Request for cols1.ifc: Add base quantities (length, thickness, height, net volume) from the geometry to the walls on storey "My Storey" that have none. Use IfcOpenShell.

First a look at what the model holds.

```python
import ifcopenshell
import ifcopenshell.util.element
import ifcopenshell.util.unit

model = ifcopenshell.open("cols1.ifc")
print(model.schema)
for unit_type in ("LENGTHUNIT", "AREAUNIT", "VOLUMEUNIT"):
    print(unit_type, ifcopenshell.util.unit.calculate_unit_scale(model, unit_type))
storey = next(s for s in model.by_type("IfcBuildingStorey") if s.Name == "My Storey")
walls = [e for e in ifcopenshell.util.element.get_decomposition(storey) if e.is_a("IfcWall")]
for e in sorted(walls, key=lambda e: e.id()):
    print(e.id(), e.is_a(), e.Name, list(ifcopenshell.util.element.get_psets(e, qtos_only=True)), sep=" | ")
```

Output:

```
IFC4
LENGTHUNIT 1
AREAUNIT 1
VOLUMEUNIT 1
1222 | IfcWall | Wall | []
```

```python
import ifcopenshell
import ifcopenshell.api.pset
import ifcopenshell.geom
import ifcopenshell.util.element
import ifcopenshell.util.shape
import ifcopenshell.util.unit

model = ifcopenshell.open("cols1.ifc")
unit_scale = ifcopenshell.util.unit.calculate_unit_scale(model)
volume_scale = ifcopenshell.util.unit.calculate_unit_scale(model, "VOLUMEUNIT")
settings = ifcopenshell.geom.settings()

storey = next(s for s in model.by_type("IfcBuildingStorey") if s.Name == "My Storey")
walls = [e for e in ifcopenshell.util.element.get_decomposition(storey) if e.is_a("IfcWall")]

for e in sorted(walls, key=lambda e: e.id()):
    if ifcopenshell.util.element.get_psets(e, qtos_only=True, should_inherit=False):
        continue
    # Geometry comes back in metres, in the element's own axes.
    shape = ifcopenshell.geom.create_shape(settings, e)
    values = {
        "Length": ifcopenshell.util.shape.get_x(shape.geometry) / unit_scale,
        "Width": ifcopenshell.util.shape.get_y(shape.geometry) / unit_scale,
        "Height": ifcopenshell.util.shape.get_z(shape.geometry) / unit_scale,
        "NetVolume": ifcopenshell.util.shape.get_volume(shape.geometry) / volume_scale,
    }
    qto = ifcopenshell.api.pset.add_qto(model, product=e, name="Qto_WallBaseQuantities")
    ifcopenshell.api.pset.edit_qto(model, qto=qto, properties=values)
    print(e.id(), {k: round(v, 3) for k, v in values.items()})

model.write("cols1-out.ifc")
```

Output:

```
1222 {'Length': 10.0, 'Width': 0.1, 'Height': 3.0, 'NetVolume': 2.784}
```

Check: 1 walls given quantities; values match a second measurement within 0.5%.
